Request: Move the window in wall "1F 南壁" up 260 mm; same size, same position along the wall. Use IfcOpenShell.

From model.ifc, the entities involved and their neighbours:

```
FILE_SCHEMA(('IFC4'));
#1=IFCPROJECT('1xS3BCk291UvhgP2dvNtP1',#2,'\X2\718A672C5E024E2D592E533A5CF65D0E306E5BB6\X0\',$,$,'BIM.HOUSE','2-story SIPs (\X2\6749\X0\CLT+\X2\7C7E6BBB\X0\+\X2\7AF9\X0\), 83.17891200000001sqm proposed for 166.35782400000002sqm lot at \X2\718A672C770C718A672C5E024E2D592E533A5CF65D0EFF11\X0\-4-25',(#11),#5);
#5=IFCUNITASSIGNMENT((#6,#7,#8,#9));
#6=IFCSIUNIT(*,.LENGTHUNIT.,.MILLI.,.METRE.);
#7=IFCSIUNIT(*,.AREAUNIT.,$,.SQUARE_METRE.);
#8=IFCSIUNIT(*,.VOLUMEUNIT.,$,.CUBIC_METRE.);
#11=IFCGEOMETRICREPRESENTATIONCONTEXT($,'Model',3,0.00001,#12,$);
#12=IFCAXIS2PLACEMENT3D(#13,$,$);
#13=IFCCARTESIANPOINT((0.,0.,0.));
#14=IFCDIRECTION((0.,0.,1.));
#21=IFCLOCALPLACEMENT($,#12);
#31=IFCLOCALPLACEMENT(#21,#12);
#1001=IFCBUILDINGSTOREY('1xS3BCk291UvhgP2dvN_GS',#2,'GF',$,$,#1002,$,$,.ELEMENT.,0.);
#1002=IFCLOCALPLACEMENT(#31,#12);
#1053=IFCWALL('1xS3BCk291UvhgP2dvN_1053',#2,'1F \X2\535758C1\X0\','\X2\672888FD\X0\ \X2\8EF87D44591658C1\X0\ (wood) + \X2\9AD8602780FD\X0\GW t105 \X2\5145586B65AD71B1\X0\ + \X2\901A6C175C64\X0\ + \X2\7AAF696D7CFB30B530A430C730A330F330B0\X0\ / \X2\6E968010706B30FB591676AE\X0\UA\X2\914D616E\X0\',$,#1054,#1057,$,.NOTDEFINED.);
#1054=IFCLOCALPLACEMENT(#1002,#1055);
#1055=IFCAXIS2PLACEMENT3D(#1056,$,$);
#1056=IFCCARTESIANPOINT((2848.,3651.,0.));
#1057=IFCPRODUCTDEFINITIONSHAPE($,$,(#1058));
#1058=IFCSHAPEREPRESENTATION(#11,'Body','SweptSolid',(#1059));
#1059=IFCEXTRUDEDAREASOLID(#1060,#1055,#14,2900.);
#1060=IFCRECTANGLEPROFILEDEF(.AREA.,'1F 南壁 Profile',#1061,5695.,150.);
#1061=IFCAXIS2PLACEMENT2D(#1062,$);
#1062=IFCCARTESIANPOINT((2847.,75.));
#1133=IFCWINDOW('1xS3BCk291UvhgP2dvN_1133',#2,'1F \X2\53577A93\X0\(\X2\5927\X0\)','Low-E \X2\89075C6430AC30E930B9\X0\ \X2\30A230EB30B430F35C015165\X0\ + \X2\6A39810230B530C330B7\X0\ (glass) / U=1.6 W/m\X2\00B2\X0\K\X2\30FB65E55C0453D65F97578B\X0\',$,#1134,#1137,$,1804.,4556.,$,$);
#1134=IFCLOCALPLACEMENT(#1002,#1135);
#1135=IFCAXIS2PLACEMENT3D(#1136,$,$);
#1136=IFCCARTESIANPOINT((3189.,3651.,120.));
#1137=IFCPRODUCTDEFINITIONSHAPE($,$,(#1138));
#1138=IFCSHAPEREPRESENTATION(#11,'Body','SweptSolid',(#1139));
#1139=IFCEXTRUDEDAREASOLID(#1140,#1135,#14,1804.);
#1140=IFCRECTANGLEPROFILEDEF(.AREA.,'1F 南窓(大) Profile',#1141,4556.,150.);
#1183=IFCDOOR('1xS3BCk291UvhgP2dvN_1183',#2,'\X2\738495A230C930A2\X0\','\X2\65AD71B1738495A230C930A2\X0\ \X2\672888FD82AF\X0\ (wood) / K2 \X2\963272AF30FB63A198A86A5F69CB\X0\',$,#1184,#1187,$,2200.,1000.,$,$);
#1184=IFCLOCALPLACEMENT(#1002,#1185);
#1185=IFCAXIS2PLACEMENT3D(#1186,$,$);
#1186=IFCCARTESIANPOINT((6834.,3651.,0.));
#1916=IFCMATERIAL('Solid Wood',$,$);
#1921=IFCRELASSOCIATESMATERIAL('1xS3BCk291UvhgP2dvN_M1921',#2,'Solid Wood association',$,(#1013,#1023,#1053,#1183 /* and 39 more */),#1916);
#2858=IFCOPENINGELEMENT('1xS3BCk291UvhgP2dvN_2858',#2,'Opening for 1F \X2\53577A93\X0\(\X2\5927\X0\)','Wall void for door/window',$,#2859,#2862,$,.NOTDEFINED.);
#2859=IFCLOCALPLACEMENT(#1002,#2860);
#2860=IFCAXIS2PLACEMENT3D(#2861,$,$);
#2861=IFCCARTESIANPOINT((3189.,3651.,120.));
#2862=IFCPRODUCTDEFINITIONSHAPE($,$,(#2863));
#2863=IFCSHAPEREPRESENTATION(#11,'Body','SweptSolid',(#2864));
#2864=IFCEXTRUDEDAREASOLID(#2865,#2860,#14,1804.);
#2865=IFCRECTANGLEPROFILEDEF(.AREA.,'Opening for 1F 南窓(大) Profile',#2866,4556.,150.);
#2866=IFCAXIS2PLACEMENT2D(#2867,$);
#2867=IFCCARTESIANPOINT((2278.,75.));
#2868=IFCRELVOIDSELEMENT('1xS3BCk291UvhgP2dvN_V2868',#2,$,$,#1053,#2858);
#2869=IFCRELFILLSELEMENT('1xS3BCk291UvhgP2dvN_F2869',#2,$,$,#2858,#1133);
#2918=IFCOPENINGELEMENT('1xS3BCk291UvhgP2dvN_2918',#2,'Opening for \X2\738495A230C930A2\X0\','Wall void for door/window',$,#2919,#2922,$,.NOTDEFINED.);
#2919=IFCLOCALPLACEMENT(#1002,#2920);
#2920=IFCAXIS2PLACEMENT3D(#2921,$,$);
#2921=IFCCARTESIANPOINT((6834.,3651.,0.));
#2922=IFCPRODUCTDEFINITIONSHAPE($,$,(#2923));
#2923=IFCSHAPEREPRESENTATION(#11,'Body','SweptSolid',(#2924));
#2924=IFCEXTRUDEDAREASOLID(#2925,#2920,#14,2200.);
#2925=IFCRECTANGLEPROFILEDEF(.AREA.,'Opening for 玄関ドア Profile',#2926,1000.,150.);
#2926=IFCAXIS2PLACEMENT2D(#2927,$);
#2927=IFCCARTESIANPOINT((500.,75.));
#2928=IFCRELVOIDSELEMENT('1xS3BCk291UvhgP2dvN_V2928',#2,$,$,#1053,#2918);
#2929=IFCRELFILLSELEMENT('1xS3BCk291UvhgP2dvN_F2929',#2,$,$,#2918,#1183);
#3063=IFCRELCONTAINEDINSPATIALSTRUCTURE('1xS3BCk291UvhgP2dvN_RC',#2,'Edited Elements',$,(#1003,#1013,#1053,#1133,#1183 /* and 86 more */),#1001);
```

```python
import numpy as np
import ifcopenshell
import ifcopenshell.api.geometry
import ifcopenshell.util.placement
import ifcopenshell.util.unit

model = ifcopenshell.open("model.ifc")
unit_scale = ifcopenshell.util.unit.calculate_unit_scale(model)

window = model.by_guid("1xS3BCk291UvhgP2dvN_1133")
opening = window.FillsVoids[0].RelatingOpeningElement
dz = 0.26 / unit_scale

shift = np.array([0.0, 0.0, dz])
# The window is not placed relative to its opening, so move both.
for product in (opening, window):
    matrix = ifcopenshell.util.placement.get_local_placement(product.ObjectPlacement)
    matrix[:3, 3] += shift
    ifcopenshell.api.geometry.edit_object_placement(model, product=product, matrix=matrix, is_si=False)

print(f"moved by {dz * unit_scale:+.3f} m")

model.write("model-out.ifc")
```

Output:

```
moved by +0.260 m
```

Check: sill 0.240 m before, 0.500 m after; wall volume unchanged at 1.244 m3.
